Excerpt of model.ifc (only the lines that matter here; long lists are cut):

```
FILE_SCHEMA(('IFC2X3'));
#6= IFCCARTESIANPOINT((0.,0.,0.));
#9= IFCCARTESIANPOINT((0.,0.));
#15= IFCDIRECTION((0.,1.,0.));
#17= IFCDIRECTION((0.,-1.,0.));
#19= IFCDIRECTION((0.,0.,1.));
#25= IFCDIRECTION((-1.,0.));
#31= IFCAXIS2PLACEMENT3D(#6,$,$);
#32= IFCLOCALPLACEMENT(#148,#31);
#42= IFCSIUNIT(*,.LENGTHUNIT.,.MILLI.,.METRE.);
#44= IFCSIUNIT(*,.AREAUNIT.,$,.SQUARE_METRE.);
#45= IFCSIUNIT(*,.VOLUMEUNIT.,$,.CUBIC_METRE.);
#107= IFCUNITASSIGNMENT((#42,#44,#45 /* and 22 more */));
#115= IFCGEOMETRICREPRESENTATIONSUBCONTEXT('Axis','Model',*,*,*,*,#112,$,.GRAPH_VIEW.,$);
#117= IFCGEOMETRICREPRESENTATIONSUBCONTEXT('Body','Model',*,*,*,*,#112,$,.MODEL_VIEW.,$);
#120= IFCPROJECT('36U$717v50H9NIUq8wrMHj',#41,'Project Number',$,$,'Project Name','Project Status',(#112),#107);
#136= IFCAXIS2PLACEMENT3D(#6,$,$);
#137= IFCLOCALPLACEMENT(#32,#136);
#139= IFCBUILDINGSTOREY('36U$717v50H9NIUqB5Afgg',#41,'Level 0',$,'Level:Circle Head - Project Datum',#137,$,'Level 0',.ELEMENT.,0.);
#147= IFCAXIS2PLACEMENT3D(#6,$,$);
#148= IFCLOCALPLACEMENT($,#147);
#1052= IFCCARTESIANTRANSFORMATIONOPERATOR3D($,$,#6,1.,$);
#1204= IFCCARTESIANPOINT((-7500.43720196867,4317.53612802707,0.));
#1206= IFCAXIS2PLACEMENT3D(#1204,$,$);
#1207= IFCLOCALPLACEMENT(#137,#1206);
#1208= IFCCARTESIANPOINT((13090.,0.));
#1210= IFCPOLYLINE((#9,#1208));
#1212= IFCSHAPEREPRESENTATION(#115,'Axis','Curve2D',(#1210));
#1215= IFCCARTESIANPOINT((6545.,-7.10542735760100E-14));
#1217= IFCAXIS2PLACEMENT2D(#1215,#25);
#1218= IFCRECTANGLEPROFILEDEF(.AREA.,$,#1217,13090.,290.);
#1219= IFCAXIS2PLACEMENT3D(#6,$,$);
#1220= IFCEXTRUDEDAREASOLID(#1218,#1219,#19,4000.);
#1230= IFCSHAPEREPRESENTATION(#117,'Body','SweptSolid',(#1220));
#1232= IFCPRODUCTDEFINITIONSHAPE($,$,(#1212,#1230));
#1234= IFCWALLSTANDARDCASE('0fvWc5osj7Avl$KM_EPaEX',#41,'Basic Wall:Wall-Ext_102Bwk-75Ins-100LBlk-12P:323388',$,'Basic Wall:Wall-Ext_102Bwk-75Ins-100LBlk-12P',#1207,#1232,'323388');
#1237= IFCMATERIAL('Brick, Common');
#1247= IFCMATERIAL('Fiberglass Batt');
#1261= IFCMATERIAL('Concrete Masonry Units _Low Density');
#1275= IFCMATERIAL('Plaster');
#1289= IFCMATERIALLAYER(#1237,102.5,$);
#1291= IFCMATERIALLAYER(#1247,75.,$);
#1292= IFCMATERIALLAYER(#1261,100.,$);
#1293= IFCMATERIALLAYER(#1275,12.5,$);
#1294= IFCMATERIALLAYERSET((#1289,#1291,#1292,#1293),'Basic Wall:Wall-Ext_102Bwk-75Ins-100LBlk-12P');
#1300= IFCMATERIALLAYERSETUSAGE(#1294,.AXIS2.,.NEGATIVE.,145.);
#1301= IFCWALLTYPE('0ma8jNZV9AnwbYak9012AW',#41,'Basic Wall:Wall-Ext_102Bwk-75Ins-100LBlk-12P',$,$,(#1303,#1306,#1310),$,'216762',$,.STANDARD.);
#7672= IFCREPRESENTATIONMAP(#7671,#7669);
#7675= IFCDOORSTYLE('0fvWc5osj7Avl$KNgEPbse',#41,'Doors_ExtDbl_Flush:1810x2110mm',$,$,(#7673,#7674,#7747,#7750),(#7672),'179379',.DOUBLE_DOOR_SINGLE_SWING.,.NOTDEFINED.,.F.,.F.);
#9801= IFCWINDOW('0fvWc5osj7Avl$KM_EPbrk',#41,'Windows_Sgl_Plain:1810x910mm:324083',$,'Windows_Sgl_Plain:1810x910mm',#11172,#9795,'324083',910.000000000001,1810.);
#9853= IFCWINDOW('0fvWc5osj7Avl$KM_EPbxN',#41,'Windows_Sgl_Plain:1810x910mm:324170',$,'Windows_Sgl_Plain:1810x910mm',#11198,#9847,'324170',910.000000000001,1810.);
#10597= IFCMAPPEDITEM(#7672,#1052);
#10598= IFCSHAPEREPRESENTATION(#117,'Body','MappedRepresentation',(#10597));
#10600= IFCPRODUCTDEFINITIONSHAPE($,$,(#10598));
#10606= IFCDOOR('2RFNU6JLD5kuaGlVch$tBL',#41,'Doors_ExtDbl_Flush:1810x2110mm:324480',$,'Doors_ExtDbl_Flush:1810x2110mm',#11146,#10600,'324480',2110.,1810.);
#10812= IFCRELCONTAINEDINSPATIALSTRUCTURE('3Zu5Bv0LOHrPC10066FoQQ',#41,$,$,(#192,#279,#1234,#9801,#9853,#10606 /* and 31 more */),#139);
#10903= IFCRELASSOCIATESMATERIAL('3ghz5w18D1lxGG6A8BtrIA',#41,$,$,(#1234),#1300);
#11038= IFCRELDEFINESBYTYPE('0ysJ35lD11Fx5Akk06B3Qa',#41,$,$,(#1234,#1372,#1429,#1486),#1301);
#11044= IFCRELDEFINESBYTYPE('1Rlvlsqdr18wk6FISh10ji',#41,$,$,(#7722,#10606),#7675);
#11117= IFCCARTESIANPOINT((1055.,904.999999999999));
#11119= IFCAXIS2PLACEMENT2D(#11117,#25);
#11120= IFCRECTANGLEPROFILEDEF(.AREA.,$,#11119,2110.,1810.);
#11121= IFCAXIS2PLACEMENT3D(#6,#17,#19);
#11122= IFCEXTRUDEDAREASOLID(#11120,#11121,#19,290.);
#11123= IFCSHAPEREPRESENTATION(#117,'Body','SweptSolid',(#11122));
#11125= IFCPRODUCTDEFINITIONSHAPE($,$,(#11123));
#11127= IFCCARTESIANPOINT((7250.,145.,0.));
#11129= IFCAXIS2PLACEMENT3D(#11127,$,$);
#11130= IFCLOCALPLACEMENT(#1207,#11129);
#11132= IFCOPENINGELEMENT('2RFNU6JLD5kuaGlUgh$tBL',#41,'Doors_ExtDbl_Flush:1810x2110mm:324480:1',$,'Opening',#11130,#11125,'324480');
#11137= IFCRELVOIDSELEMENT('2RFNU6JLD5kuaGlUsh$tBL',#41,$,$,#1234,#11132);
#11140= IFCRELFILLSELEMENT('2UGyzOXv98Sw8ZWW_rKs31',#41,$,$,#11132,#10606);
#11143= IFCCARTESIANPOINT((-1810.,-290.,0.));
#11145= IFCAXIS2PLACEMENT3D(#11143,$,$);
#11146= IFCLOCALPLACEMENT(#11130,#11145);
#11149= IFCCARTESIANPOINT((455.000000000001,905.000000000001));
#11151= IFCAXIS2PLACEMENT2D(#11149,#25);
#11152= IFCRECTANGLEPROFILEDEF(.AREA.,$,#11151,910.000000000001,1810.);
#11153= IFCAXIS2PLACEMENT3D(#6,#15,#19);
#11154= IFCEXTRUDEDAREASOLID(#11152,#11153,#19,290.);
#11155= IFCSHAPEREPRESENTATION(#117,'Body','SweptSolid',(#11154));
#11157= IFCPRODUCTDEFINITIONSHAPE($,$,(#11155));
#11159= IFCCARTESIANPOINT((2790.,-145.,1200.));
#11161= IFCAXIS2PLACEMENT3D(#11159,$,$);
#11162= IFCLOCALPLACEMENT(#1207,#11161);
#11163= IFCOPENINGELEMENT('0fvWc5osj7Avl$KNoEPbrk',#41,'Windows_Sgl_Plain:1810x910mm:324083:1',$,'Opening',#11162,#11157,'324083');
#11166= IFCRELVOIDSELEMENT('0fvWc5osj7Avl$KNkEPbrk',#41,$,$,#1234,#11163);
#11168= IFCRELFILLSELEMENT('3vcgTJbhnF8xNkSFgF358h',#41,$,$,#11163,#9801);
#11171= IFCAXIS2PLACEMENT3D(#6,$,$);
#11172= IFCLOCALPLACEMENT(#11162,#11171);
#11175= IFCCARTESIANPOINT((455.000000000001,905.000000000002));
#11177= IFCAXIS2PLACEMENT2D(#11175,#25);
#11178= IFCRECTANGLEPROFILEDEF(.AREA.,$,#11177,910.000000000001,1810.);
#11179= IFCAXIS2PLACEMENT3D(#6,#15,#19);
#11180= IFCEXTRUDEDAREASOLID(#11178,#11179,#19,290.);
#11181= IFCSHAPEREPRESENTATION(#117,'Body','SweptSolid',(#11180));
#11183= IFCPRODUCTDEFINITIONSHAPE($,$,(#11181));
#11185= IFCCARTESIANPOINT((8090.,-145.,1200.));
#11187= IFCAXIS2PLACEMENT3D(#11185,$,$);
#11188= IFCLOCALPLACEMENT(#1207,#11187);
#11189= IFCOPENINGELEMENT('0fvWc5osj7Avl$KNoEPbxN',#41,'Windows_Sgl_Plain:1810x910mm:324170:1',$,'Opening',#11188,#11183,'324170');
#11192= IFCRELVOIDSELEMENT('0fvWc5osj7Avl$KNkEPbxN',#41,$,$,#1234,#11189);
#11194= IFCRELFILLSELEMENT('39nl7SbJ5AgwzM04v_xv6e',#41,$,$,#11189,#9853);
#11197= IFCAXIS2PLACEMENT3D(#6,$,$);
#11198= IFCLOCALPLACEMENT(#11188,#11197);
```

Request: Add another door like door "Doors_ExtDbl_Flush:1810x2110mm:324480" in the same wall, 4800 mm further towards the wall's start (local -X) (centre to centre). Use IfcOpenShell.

```python
import ifcopenshell
import ifcopenshell.api.feature
import ifcopenshell.api.geometry
import ifcopenshell.api.root
import ifcopenshell.geom
import ifcopenshell.util.element
import ifcopenshell.util.placement
import ifcopenshell.util.shape
import ifcopenshell.util.unit

model = ifcopenshell.open("model.ifc")
unit_scale = ifcopenshell.util.unit.calculate_unit_scale(model)
settings = ifcopenshell.geom.settings()


def volume(element):
    """Net volume in cubic metres, openings subtracted."""
    shape = ifcopenshell.geom.create_shape(settings, element)
    return ifcopenshell.util.shape.get_volume(shape.geometry)


def reuse_history(source, copy):
    """copy_class also copies each property set's owner history, people and application; keep the originals."""
    for rel in copy.IsDefinedBy:
        if rel.is_a("IfcRelDefinesByProperties") and (history := rel.RelatingPropertyDefinition.OwnerHistory):
            rel.RelatingPropertyDefinition.OwnerHistory = source.OwnerHistory
            ifcopenshell.util.element.remove_deep2(model, history)


door = model.by_guid("2RFNU6JLD5kuaGlVch$tBL")
opening = door.FillsVoids[0].RelatingOpeningElement
wall = opening.VoidsElements[0].RelatingBuildingElement
before = volume(wall)
shift = ifcopenshell.util.placement.get_local_placement(wall.ObjectPlacement)[:3, 0] * -4.8 / unit_scale

# copy_class copies the void relationship, type, container and properties, but no geometry.
new_opening = ifcopenshell.api.root.copy_class(model, product=opening)
new_opening.Representation = ifcopenshell.util.element.copy_deep(
    model, opening.Representation, exclude=["IfcGeometricRepresentationContext", "IfcRepresentationMap"]
)
new_opening.Name = "Doors_ExtDbl_Flush:1810x2110mm"
new_opening.Tag = None
new_door = ifcopenshell.api.root.copy_class(model, product=door)
new_door.Representation = ifcopenshell.util.element.copy_deep(
    model, door.Representation, exclude=["IfcGeometricRepresentationContext", "IfcRepresentationMap"]
)
new_door.Name = "Doors_ExtDbl_Flush:1810x2110mm"
new_door.Tag = None
reuse_history(door, new_door)
fills = ifcopenshell.api.feature.add_filling(model, opening=new_opening, element=new_door)
fills.OwnerHistory = new_door.OwnerHistory  # required in IFC2X3

for old, new in ((opening, new_opening), (door, new_door)):
    matrix = ifcopenshell.util.placement.get_local_placement(old.ObjectPlacement)
    matrix[:3, 3] += shift
    ifcopenshell.api.geometry.edit_object_placement(model, product=new, matrix=matrix, is_si=False)

after = volume(wall)

print(f"wall volume {before:.3f} -> {after:.3f} m3")

model.write("model_rev.ifc")
```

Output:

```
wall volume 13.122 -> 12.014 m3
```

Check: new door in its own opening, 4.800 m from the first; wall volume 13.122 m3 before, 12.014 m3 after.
